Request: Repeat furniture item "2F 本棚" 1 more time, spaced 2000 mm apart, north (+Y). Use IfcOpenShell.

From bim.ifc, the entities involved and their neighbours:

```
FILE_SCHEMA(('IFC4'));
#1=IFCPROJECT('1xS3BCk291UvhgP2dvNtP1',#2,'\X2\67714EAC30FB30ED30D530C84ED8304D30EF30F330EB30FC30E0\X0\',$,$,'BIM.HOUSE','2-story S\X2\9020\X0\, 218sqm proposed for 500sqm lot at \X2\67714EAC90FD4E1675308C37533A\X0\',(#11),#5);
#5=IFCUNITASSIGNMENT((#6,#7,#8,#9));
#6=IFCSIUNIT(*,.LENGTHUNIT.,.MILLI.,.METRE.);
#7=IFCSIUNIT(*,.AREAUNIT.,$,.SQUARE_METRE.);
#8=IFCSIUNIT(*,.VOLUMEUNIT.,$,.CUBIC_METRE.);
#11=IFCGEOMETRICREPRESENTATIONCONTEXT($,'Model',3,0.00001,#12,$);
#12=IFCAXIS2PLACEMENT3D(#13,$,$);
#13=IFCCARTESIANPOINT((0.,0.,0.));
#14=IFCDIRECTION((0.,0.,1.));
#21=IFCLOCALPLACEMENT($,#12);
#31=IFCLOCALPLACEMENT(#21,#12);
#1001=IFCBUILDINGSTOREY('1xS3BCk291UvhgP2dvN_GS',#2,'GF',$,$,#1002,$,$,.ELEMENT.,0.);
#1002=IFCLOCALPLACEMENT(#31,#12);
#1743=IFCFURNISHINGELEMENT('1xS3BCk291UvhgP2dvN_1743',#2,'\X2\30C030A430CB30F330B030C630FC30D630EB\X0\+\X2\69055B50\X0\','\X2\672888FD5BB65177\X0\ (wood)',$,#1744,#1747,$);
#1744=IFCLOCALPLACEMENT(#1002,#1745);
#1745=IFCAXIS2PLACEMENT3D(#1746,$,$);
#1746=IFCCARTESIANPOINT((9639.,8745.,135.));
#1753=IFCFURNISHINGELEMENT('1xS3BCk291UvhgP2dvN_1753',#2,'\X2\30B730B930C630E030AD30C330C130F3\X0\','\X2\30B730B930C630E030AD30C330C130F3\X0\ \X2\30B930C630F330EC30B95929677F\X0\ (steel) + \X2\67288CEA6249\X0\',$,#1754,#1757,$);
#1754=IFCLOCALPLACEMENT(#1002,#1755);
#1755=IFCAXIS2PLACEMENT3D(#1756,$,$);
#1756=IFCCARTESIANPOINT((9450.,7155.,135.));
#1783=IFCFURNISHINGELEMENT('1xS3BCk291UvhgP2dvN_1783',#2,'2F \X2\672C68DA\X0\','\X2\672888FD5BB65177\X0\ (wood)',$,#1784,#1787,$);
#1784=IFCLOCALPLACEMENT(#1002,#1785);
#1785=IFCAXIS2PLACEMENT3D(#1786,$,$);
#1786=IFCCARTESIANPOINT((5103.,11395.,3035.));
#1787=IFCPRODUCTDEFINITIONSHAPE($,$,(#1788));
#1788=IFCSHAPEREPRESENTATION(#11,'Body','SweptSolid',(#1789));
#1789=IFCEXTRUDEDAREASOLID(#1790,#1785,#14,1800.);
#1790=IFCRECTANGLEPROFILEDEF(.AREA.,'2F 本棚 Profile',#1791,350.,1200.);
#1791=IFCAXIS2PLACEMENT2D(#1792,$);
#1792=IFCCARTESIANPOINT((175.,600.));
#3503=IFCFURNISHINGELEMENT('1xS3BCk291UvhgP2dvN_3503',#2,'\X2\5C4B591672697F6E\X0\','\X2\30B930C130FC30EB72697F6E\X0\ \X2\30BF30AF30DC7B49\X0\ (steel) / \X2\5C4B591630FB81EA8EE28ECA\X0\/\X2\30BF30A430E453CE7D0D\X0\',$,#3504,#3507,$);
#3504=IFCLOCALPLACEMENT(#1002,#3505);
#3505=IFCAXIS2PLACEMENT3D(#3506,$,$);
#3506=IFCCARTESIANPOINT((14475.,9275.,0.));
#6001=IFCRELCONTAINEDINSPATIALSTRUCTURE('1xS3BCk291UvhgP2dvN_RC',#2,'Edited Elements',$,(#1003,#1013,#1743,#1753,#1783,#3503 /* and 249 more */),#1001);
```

```python
import numpy as np
import ifcopenshell
import ifcopenshell.api.geometry
import ifcopenshell.api.root
import ifcopenshell.util.element
import ifcopenshell.util.placement
import ifcopenshell.util.unit

model = ifcopenshell.open("bim.ifc")
unit_scale = ifcopenshell.util.unit.calculate_unit_scale(model)


def reuse_history(source, copy):
    """copy_class also copies each property set's owner history, people and application; keep the originals."""
    for rel in copy.IsDefinedBy:
        if rel.is_a("IfcRelDefinesByProperties") and (history := rel.RelatingPropertyDefinition.OwnerHistory):
            rel.RelatingPropertyDefinition.OwnerHistory = source.OwnerHistory
            ifcopenshell.util.element.remove_deep2(model, history)


source = model.by_guid("1xS3BCk291UvhgP2dvN_1783")
base = ifcopenshell.util.placement.get_local_placement(source.ObjectPlacement)
step = np.array([0.0, 1.0, 0.0]) * 2 / unit_scale

for i in range(1, 2):
    copy = ifcopenshell.api.root.copy_class(model, product=source)
    copy.Representation = ifcopenshell.util.element.copy_deep(
        model, source.Representation, exclude=["IfcGeometricRepresentationContext", "IfcRepresentationMap"]
    )
    reuse_history(source, copy)
    matrix = base.copy()
    matrix[:3, 3] += i * step
    print("added at", matrix[:3, 3].round(3) + 0.0)
    ifcopenshell.api.geometry.edit_object_placement(model, product=copy, matrix=matrix, is_si=False)

model.write("bim_edited.ifc")
```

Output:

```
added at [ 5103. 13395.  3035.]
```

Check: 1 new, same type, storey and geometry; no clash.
